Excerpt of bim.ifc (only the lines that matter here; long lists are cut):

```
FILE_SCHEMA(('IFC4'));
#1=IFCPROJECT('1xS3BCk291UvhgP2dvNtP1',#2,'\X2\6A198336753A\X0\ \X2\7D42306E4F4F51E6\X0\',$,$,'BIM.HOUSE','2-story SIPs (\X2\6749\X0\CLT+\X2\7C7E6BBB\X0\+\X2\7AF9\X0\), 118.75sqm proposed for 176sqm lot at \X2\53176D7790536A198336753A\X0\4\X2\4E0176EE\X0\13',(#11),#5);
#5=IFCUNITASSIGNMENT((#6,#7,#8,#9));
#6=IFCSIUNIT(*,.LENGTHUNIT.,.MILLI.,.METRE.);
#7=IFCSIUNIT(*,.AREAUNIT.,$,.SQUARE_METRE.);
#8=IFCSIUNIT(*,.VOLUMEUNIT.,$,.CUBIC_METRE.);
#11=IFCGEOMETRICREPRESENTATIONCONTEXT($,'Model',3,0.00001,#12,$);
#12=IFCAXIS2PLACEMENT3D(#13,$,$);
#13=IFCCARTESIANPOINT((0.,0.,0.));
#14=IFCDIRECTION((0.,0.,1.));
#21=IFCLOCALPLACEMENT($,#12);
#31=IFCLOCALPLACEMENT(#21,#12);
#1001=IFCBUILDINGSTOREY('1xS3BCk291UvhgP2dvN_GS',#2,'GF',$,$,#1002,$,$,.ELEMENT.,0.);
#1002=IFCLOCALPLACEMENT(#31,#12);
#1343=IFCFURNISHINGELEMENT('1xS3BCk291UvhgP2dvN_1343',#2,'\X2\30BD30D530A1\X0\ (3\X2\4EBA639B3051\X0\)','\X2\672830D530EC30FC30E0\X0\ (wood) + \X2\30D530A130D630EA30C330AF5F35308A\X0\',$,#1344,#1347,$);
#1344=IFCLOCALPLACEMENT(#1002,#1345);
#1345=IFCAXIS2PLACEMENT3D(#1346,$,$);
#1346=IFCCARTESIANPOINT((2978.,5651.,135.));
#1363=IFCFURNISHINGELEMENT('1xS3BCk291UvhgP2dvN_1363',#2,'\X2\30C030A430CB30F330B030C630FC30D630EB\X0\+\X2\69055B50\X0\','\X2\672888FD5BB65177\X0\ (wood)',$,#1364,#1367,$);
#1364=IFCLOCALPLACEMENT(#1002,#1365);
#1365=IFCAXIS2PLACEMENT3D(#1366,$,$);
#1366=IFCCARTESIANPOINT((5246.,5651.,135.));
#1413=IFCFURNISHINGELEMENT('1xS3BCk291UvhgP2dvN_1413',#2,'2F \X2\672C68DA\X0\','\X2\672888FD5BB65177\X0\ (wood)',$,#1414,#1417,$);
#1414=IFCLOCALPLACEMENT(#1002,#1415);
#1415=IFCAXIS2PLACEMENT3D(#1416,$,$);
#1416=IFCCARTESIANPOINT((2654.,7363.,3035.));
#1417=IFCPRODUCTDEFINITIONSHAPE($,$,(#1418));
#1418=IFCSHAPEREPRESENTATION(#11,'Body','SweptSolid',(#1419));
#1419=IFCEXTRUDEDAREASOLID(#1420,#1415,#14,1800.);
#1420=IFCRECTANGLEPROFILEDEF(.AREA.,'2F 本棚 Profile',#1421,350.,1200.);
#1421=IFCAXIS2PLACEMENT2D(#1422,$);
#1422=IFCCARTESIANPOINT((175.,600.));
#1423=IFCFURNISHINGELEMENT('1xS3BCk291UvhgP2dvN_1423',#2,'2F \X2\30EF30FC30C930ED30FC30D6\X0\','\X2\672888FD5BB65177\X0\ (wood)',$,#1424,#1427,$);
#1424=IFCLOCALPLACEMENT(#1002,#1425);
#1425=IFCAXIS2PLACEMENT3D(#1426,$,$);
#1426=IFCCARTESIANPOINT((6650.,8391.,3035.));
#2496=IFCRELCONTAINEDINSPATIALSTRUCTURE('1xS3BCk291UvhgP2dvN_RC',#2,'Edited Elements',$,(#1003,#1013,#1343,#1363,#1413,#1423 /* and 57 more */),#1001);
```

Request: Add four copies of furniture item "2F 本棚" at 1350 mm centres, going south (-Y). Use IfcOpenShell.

```python
import numpy as np
import ifcopenshell
import ifcopenshell.api.geometry
import ifcopenshell.api.root
import ifcopenshell.util.element
import ifcopenshell.util.placement

model = ifcopenshell.open("bim.ifc")


def reuse_history(source, copy):
    """copy_class also copies each property set's owner history, people and application; keep the originals."""
    for rel in copy.IsDefinedBy:
        if rel.is_a("IfcRelDefinesByProperties") and (history := rel.RelatingPropertyDefinition.OwnerHistory):
            rel.RelatingPropertyDefinition.OwnerHistory = source.OwnerHistory
            ifcopenshell.util.element.remove_deep2(model, history)


source = model.by_id(1413)
base = ifcopenshell.util.placement.get_local_placement(source.ObjectPlacement)
step = np.array([0.0, -1.0, 0.0]) * 1350.0

for i in range(1, 5):
    copy = ifcopenshell.api.root.copy_class(model, product=source)
    copy.Representation = ifcopenshell.util.element.copy_deep(
        model, source.Representation, exclude=["IfcGeometricRepresentationContext", "IfcRepresentationMap"]
    )
    reuse_history(source, copy)
    matrix = base.copy()
    matrix[:3, 3] += i * step
    print("added at", matrix[:3, 3].round(3) + 0.0)
    ifcopenshell.api.geometry.edit_object_placement(model, product=copy, matrix=matrix, is_si=False)

model.write("bim_edited.ifc")
```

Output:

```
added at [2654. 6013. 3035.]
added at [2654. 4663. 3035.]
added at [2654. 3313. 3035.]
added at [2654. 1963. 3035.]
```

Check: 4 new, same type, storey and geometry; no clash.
